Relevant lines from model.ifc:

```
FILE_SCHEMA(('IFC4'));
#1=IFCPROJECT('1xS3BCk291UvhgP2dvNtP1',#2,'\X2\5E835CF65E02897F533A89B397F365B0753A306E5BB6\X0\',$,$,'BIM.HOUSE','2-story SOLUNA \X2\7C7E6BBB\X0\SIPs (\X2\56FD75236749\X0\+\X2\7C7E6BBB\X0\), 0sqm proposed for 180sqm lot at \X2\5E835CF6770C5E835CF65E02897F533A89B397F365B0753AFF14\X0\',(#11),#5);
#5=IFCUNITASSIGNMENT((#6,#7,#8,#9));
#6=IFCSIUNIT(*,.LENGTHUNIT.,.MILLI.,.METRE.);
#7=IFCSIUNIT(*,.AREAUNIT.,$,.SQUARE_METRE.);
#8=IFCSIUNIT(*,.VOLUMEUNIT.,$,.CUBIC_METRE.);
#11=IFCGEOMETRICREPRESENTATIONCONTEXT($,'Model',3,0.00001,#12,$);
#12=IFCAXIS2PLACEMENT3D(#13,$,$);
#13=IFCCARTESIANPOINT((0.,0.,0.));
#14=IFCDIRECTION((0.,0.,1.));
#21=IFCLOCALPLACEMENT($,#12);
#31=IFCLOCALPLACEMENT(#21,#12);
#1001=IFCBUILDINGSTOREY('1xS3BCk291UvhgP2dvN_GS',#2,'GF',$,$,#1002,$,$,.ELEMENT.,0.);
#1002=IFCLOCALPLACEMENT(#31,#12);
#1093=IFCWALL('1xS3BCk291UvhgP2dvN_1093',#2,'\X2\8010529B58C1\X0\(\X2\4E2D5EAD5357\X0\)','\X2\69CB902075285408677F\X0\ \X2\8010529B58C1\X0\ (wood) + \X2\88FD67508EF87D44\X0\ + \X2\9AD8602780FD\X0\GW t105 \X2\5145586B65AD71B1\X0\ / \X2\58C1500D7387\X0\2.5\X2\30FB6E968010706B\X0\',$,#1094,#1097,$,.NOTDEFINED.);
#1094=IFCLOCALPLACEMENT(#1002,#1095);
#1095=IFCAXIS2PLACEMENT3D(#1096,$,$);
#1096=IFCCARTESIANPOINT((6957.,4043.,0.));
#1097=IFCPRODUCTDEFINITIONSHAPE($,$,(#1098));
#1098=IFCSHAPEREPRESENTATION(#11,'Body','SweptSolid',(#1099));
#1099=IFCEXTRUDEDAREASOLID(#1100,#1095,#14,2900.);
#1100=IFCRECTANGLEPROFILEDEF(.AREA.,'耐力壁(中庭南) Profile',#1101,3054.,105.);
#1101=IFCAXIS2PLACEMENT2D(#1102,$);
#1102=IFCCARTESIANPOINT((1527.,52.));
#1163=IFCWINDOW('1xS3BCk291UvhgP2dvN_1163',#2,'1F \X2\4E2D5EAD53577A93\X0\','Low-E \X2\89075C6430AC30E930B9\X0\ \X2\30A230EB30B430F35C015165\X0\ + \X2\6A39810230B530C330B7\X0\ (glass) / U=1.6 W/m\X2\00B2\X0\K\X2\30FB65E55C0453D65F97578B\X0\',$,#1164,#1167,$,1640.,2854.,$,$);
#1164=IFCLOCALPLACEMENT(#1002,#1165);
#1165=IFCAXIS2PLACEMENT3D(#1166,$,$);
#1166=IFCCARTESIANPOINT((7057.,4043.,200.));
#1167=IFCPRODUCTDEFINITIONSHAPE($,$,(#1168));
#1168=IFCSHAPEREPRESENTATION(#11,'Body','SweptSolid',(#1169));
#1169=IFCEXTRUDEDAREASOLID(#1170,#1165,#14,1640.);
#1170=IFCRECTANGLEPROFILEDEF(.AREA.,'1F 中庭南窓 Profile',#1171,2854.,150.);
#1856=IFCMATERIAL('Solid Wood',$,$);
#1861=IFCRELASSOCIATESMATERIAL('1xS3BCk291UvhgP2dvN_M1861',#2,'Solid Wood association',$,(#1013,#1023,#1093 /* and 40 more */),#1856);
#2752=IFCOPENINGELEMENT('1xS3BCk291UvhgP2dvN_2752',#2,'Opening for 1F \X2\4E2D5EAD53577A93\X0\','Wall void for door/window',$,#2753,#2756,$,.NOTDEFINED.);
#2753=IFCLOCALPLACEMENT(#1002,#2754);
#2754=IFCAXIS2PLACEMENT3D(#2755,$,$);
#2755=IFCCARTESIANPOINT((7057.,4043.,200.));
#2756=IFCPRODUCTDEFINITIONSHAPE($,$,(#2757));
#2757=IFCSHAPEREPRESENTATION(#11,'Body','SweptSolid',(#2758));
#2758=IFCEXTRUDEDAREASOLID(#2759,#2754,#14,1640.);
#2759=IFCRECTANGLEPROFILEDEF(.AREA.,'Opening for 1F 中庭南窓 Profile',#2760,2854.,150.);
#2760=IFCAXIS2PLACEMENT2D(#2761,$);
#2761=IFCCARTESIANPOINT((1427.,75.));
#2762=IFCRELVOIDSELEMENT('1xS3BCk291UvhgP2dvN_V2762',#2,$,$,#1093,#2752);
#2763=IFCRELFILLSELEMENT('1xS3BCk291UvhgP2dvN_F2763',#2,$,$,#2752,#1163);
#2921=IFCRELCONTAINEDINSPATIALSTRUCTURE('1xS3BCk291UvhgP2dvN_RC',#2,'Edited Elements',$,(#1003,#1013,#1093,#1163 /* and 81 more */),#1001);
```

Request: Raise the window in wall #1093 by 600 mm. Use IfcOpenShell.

```python
import numpy as np
import ifcopenshell
import ifcopenshell.api.geometry
import ifcopenshell.util.placement
import ifcopenshell.util.unit

model = ifcopenshell.open("model.ifc")
unit_scale = ifcopenshell.util.unit.calculate_unit_scale(model)

window = model.by_guid("1xS3BCk291UvhgP2dvN_1163")
opening = window.FillsVoids[0].RelatingOpeningElement
dz = 600.0

shift = np.array([0.0, 0.0, dz])
# The window is not placed relative to its opening, so move both.
for product in (opening, window):
    matrix = ifcopenshell.util.placement.get_local_placement(product.ObjectPlacement)
    matrix[:3, 3] += shift
    ifcopenshell.api.geometry.edit_object_placement(model, product=product, matrix=matrix, is_si=False)

print(f"moved by {dz * unit_scale:+.3f} m")

model.write("model_updated.ifc")
```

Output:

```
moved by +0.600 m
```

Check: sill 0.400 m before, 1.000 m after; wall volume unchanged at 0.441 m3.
